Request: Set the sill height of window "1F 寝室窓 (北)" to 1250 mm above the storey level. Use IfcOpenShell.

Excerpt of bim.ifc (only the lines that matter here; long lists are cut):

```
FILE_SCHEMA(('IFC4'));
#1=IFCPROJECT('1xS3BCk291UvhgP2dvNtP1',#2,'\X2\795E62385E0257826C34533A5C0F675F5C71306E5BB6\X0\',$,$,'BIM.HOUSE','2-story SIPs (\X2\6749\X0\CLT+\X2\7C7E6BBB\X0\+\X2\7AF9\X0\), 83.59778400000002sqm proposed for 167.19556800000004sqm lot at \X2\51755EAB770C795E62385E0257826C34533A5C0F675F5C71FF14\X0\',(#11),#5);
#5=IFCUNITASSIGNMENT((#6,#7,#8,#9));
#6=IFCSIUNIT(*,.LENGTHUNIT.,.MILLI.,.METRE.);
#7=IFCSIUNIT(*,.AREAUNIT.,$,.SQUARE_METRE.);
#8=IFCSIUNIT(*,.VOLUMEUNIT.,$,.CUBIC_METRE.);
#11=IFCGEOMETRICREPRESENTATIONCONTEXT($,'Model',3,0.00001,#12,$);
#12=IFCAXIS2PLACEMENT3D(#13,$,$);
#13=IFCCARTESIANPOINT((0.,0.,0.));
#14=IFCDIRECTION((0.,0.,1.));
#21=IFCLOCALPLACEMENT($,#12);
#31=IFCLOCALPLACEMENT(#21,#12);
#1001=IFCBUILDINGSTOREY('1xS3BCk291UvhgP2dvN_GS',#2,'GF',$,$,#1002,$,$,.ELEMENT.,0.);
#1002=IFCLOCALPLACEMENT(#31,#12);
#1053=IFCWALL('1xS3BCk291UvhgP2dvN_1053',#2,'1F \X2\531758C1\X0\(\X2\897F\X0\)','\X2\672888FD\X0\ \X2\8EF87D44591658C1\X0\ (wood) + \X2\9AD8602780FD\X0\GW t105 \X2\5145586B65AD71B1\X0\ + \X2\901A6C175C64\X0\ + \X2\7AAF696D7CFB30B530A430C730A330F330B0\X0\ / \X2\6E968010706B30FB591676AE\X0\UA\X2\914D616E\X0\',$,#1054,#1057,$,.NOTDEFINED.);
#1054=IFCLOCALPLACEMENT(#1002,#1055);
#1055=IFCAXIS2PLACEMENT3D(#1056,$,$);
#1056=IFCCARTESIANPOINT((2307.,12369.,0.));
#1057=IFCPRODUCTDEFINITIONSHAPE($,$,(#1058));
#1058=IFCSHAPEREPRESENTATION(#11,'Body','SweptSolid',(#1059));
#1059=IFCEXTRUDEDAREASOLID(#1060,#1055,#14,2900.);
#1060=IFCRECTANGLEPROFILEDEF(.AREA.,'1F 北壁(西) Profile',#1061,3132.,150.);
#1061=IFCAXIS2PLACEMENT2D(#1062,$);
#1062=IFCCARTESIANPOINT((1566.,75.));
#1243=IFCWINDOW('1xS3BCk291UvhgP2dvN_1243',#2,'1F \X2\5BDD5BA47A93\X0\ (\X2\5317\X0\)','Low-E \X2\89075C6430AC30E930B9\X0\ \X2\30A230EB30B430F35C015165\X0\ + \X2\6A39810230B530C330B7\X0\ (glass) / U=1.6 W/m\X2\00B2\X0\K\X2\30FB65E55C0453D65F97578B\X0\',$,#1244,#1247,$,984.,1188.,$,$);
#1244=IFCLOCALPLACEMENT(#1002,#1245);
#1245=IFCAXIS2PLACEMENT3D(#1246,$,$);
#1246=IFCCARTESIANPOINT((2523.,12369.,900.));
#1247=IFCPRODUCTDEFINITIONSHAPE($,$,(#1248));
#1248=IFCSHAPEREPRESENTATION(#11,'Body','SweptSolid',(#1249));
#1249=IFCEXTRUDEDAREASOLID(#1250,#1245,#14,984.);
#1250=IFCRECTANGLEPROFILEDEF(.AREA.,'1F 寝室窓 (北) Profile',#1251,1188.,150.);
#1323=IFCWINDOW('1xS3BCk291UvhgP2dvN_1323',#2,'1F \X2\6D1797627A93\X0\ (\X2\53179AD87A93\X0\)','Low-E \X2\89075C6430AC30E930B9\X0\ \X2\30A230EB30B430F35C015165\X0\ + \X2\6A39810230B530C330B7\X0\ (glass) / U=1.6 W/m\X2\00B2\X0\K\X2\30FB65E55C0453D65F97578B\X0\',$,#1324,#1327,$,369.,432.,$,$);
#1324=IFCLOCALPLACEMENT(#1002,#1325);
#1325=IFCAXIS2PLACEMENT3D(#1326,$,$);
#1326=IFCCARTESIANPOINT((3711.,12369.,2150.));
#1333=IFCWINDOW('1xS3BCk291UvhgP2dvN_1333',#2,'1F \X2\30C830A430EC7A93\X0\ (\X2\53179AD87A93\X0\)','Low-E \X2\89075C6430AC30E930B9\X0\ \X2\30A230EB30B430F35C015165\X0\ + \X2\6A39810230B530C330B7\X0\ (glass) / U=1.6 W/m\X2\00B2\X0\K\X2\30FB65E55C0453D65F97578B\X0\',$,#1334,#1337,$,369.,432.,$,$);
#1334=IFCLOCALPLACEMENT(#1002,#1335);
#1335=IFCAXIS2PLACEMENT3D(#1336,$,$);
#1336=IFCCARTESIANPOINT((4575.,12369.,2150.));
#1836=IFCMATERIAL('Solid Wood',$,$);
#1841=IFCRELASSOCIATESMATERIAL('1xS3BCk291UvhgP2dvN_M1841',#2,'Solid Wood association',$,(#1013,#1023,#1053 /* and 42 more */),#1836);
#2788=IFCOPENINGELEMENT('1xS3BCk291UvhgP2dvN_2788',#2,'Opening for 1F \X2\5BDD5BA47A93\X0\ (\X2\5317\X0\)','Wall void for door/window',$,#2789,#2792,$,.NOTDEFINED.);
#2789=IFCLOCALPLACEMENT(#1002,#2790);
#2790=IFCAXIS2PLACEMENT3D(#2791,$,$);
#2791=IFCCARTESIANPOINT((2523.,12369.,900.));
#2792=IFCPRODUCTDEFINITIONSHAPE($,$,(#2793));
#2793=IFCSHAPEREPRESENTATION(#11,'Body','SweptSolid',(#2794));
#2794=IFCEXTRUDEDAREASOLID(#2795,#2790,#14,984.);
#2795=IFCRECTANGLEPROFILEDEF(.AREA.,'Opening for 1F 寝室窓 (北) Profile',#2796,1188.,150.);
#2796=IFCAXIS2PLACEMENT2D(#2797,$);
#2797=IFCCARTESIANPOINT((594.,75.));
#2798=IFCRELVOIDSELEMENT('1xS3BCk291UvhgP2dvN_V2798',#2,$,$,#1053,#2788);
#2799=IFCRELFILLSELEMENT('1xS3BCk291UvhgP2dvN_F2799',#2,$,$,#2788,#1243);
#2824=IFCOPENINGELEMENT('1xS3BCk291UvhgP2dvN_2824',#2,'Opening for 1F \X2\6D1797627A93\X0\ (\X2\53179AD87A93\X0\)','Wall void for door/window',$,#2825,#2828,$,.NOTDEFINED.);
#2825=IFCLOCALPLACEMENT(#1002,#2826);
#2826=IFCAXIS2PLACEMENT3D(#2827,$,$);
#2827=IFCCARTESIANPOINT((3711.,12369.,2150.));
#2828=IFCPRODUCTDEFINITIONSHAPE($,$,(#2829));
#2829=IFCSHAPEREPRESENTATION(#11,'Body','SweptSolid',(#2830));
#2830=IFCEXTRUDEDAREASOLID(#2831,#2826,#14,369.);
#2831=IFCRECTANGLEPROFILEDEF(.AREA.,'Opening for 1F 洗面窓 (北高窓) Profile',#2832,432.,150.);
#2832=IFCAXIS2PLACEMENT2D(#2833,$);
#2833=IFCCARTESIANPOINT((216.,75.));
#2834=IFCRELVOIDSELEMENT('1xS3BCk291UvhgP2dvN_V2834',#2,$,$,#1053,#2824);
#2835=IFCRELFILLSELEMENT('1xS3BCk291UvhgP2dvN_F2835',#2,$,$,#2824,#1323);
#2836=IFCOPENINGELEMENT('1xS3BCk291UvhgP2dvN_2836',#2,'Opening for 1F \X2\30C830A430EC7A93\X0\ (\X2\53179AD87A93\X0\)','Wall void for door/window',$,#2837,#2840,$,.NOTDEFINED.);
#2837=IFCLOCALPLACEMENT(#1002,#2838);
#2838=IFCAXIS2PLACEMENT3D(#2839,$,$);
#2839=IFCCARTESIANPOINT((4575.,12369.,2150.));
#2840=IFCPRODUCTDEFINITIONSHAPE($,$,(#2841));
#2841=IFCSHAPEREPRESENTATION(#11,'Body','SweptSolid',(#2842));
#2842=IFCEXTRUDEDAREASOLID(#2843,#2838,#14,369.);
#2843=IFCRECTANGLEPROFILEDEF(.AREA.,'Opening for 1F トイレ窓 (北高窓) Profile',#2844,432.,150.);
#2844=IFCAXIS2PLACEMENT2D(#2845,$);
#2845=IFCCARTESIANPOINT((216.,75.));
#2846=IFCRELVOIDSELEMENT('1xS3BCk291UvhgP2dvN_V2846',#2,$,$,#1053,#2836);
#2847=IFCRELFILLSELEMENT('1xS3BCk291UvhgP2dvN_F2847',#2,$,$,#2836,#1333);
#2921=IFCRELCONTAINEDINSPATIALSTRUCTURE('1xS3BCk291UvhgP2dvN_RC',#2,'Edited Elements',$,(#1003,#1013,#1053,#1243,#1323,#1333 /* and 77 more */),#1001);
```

```python
import numpy as np
import ifcopenshell
import ifcopenshell.api.geometry
import ifcopenshell.geom
import ifcopenshell.util.element
import ifcopenshell.util.placement
import ifcopenshell.util.shape
import ifcopenshell.util.unit

model = ifcopenshell.open("bim.ifc")
unit_scale = ifcopenshell.util.unit.calculate_unit_scale(model)

window = model.by_id(1243)
opening = window.FillsVoids[0].RelatingOpeningElement
storey = ifcopenshell.util.element.get_container(window, ifc_class="IfcBuildingStorey")
level = ifcopenshell.util.placement.get_local_placement(storey.ObjectPlacement)[2, 3]

# The opening's origin need not be at the sill, so measure its lowest point.
shape = ifcopenshell.geom.create_shape(ifcopenshell.geom.settings(), opening)
bottom = ifcopenshell.util.shape.get_shape_bottom_elevation(shape, shape.geometry) / unit_scale
dz = level + 1.25 / unit_scale - bottom

shift = np.array([0.0, 0.0, dz])
# The window is not placed relative to its opening, so move both.
for product in (opening, window):
    matrix = ifcopenshell.util.placement.get_local_placement(product.ObjectPlacement)
    matrix[:3, 3] += shift
    ifcopenshell.api.geometry.edit_object_placement(model, product=product, matrix=matrix, is_si=False)

print(f"moved by {dz * unit_scale:+.3f} m")

model.write("bim-out.ifc")
```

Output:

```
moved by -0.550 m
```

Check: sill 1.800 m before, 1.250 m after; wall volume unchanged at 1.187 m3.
